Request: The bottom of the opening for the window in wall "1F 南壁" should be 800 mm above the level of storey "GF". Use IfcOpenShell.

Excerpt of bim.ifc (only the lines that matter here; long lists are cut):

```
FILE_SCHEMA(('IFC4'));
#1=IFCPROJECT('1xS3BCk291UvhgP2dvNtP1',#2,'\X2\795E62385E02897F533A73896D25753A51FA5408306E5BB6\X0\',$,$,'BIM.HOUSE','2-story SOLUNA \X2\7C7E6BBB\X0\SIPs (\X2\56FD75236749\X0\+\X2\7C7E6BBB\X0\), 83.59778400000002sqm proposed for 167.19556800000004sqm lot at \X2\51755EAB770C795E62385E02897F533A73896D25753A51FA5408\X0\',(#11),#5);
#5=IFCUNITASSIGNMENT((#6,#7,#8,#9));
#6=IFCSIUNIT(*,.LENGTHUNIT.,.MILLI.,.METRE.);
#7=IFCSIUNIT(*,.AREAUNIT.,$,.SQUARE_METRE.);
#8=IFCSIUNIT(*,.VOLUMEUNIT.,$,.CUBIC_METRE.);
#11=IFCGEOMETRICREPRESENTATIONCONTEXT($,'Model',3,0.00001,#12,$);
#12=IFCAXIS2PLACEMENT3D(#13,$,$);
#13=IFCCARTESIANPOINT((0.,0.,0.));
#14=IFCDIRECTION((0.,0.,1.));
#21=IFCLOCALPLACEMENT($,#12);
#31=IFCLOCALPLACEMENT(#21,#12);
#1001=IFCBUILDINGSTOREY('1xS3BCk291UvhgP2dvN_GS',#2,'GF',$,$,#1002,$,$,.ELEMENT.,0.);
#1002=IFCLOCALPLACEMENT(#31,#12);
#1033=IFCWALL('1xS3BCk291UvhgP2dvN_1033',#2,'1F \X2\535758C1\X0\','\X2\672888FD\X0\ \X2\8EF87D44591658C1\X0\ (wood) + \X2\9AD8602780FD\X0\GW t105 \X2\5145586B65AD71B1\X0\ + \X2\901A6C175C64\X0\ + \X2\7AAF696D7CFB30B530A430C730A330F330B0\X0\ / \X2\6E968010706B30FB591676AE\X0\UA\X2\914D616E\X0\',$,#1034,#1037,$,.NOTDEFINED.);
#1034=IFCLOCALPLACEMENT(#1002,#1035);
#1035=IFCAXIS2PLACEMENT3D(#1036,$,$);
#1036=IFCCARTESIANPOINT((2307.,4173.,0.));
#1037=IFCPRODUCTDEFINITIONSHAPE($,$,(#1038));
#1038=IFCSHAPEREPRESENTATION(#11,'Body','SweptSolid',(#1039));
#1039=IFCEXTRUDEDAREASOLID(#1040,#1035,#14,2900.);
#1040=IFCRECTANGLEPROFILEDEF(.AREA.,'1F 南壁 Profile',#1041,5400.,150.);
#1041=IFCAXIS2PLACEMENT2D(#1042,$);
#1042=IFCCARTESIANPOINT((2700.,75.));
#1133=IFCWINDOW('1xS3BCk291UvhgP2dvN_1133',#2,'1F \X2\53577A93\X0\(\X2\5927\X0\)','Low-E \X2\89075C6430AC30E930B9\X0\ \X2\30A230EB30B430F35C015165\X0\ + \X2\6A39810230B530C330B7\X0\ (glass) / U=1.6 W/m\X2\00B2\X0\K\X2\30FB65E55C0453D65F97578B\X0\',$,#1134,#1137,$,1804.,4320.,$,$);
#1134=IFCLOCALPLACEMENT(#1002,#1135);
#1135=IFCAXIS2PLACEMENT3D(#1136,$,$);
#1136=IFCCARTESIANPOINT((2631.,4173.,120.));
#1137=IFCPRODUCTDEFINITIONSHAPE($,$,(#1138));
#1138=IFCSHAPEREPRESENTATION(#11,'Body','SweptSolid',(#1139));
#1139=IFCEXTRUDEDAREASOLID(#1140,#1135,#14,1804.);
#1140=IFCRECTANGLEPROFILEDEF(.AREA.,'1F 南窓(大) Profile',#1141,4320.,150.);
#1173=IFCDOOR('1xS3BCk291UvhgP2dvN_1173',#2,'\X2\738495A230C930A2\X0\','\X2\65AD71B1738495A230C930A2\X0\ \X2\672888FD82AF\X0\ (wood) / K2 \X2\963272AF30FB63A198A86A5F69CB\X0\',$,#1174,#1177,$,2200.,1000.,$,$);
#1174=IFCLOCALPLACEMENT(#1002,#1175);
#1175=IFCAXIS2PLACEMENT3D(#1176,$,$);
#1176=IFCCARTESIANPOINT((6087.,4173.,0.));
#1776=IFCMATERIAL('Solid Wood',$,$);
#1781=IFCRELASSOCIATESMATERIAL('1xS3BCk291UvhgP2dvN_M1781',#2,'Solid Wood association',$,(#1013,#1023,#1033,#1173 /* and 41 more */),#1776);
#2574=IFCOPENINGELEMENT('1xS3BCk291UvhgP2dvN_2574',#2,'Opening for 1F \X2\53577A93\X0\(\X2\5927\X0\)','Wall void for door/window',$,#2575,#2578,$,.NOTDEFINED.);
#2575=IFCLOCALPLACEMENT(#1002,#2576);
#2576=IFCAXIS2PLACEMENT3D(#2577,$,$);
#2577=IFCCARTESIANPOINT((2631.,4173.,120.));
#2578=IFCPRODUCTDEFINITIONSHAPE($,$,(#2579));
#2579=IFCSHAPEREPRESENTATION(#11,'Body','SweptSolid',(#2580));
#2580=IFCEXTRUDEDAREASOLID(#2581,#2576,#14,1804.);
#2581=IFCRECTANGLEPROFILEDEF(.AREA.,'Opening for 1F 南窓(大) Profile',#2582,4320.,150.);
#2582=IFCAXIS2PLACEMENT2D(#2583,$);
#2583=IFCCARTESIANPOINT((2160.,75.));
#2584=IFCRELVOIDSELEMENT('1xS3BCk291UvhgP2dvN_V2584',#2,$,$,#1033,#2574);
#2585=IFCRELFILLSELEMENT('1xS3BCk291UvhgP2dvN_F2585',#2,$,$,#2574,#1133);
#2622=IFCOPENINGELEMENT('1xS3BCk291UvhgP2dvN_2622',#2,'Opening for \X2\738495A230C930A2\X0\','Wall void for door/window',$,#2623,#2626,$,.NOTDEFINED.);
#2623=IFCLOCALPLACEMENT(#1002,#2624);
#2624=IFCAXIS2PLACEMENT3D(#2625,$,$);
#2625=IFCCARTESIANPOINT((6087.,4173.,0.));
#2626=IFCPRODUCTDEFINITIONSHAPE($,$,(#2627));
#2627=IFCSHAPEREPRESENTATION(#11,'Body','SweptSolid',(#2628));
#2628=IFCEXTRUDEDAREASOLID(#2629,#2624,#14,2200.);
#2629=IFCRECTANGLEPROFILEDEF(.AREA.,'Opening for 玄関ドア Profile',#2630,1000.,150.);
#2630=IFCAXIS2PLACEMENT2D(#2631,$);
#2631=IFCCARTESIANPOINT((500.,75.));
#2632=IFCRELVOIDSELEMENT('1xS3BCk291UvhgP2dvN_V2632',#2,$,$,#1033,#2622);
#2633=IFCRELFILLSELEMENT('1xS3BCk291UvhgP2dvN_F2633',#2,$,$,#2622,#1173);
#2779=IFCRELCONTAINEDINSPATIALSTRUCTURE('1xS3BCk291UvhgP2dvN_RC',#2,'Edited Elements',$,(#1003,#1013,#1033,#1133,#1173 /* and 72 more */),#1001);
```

```python
import numpy as np
import ifcopenshell
import ifcopenshell.api.geometry
import ifcopenshell.geom
import ifcopenshell.util.element
import ifcopenshell.util.placement
import ifcopenshell.util.shape
import ifcopenshell.util.unit

model = ifcopenshell.open("bim.ifc")
unit_scale = ifcopenshell.util.unit.calculate_unit_scale(model)

window = model.by_guid("1xS3BCk291UvhgP2dvN_1133")
opening = window.FillsVoids[0].RelatingOpeningElement
storey = ifcopenshell.util.element.get_container(window, ifc_class="IfcBuildingStorey")
level = ifcopenshell.util.placement.get_local_placement(storey.ObjectPlacement)[2, 3]

# The opening's origin need not be at the sill, so measure its lowest point.
shape = ifcopenshell.geom.create_shape(ifcopenshell.geom.settings(), opening)
bottom = ifcopenshell.util.shape.get_shape_bottom_elevation(shape, shape.geometry) / unit_scale
dz = level + 800.0 - bottom

shift = np.array([0.0, 0.0, dz])
# The window is not placed relative to its opening, so move both.
for product in (opening, window):
    matrix = ifcopenshell.util.placement.get_local_placement(product.ObjectPlacement)
    matrix[:3, 3] += shift
    ifcopenshell.api.geometry.edit_object_placement(model, product=product, matrix=matrix, is_si=False)

print(f"moved by {dz * unit_scale:+.3f} m")

model.write("bim_rev.ifc")
```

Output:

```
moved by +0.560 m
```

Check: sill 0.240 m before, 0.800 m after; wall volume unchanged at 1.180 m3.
